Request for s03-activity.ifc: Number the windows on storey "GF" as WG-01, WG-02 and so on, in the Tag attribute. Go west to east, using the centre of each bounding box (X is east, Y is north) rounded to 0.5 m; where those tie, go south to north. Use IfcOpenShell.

First a look at what the model holds.

```python
import ifcopenshell
import ifcopenshell.util.element
import ifcopenshell.util.placement

model = ifcopenshell.open("s03-activity.ifc")
print(model.schema)
storey = next(s for s in model.by_type("IfcBuildingStorey") if s.Name == "GF")
windows = [e for e in ifcopenshell.util.element.get_decomposition(storey) if e.is_a("IfcWindow")]
for e in sorted(windows, key=lambda e: e.id()):
    origin = ifcopenshell.util.placement.get_local_placement(e.ObjectPlacement)[:3, 3]
    print(e.id(), e.Tag, e.Name, origin.round(2) + 0.0, sep=" | ")
```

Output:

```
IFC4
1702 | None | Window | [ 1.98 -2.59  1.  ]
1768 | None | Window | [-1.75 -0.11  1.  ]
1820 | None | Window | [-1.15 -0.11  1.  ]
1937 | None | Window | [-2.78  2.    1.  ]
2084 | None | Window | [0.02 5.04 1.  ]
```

```python
import ifcopenshell
import ifcopenshell.geom
import ifcopenshell.util.element
import ifcopenshell.util.shape

model = ifcopenshell.open("s03-activity.ifc")
settings = ifcopenshell.geom.settings()
settings.set("use-world-coords", True)


def centre(element):
    shape = ifcopenshell.geom.create_shape(settings, element)
    return ifcopenshell.util.shape.get_bbox_centroid(shape.geometry)


storey = next(s for s in model.by_type("IfcBuildingStorey") if s.Name == "GF")
windows = [e for e in ifcopenshell.util.element.get_decomposition(storey) if e.is_a("IfcWindow")]

# Insertion points can sit at a corner or the storey origin, so sort by the geometry (in metres).
centres = {e: centre(e) for e in windows}
windows.sort(key=lambda e: (round(centres[e][0] / 0.5), centres[e][1]))

for i, e in enumerate(windows, start=1):
    number = f"WG-{i:02d}"
    e.Tag = number
    print(e.id(), number)

model.write("s03-activity_updated.ifc")
```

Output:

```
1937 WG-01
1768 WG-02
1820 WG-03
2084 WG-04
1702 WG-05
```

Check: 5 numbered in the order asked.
